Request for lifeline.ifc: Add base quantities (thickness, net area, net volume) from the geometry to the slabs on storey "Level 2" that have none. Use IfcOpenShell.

First a look at what the model holds.

```python
import ifcopenshell
import ifcopenshell.util.element
import ifcopenshell.util.unit

model = ifcopenshell.open("lifeline.ifc")
print(model.schema)
for unit_type in ("LENGTHUNIT", "AREAUNIT", "VOLUMEUNIT"):
    print(unit_type, ifcopenshell.util.unit.calculate_unit_scale(model, unit_type))
storey = next(s for s in model.by_type("IfcBuildingStorey") if s.Name == "Level 2")
slabs = [e for e in ifcopenshell.util.element.get_decomposition(storey) if e.is_a("IfcSlab")]
for e in sorted(slabs, key=lambda e: e.id()):
    print(e.id(), e.is_a(), e.Name, list(ifcopenshell.util.element.get_psets(e, qtos_only=True)), sep=" | ")
```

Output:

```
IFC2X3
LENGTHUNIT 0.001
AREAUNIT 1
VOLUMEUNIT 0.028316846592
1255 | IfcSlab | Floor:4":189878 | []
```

```python
import ifcopenshell
import ifcopenshell.api.pset
import ifcopenshell.geom
import ifcopenshell.util.element
import ifcopenshell.util.shape
import ifcopenshell.util.unit

model = ifcopenshell.open("lifeline.ifc")
unit_scale = ifcopenshell.util.unit.calculate_unit_scale(model)
area_scale = ifcopenshell.util.unit.calculate_unit_scale(model, "AREAUNIT")
volume_scale = ifcopenshell.util.unit.calculate_unit_scale(model, "VOLUMEUNIT")
settings = ifcopenshell.geom.settings()

storey = next(s for s in model.by_type("IfcBuildingStorey") if s.Name == "Level 2")
slabs = [e for e in ifcopenshell.util.element.get_decomposition(storey) if e.is_a("IfcSlab")]

for e in sorted(slabs, key=lambda e: e.id()):
    if ifcopenshell.util.element.get_psets(e, qtos_only=True, should_inherit=False):
        continue
    # Geometry comes back in metres, in the element's own axes.
    shape = ifcopenshell.geom.create_shape(settings, e)
    values = {
        "Width": ifcopenshell.util.shape.get_z(shape.geometry) / unit_scale,
        "NetArea": ifcopenshell.util.shape.get_footprint_area(shape.geometry) / area_scale,
        "NetVolume": ifcopenshell.util.shape.get_volume(shape.geometry) / volume_scale,
    }
    qto = ifcopenshell.api.pset.add_qto(model, product=e, name="BaseQuantities")
    ifcopenshell.api.pset.edit_qto(model, qto=qto, properties=values)
    print(e.id(), {k: round(v, 3) for k, v in values.items()})

model.write("lifeline_rev.ifc")
```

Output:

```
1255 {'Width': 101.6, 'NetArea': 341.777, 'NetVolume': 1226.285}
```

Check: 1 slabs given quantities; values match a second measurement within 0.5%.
